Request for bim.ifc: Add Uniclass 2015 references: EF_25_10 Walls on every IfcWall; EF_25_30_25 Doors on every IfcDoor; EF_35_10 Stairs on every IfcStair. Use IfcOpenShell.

First a look at what the model holds.

```python
import ifcopenshell

model = ifcopenshell.open("bim.ifc")
print(model.schema)
print("classifications:", [c.Name for c in model.by_type("IfcClassification")])
for ifc_class in ("IfcDoor", "IfcRoof", "IfcStair", "IfcWall", "IfcWindow"):
    print(ifc_class, len(model.by_type(ifc_class)))
```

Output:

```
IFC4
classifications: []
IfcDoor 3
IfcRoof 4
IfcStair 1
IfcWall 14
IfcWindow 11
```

```python
import ifcopenshell
import ifcopenshell.api.classification

model = ifcopenshell.open("bim.ifc")

system = ifcopenshell.api.classification.add_classification(model, classification="Uniclass 2015")

codes = {
    "IfcWall": ("EF_25_10", "Walls"),
    "IfcDoor": ("EF_25_30_25", "Doors"),
    "IfcStair": ("EF_35_10", "Stairs"),
}
for ifc_class, (code, name) in codes.items():
    products = model.by_type(ifc_class)
    ifcopenshell.api.classification.add_reference(
        model, products=products, classification=system, identification=code, name=name
    )
    print(code, len(products))

model.write("bim-out.ifc")
```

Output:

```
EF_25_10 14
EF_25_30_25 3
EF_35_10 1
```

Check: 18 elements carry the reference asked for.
